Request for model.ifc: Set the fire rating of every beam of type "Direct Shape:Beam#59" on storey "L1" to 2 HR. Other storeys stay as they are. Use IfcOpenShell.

First a look at what the model holds.

```python
import ifcopenshell
import ifcopenshell.util.element

model = ifcopenshell.open("model.ifc")
print(model.schema)
storey = next(s for s in model.by_type("IfcBuildingStorey") if s.Name == "L1")
beams = [e for e in ifcopenshell.util.element.get_decomposition(storey) if e.is_a("IfcBeam")]
seen = {}
for e in beams:
    element_type = ifcopenshell.util.element.get_type(e)
    key = (element_type.Name if element_type != e and element_type else None, ifcopenshell.util.element.get_pset(e, "Pset_BeamCommon", "FireRating"))
    seen[key] = seen.get(key, 0) + 1
for (name, value), count in sorted(seen.items(), key=str):
    print(count, "x", name, "|", value)
```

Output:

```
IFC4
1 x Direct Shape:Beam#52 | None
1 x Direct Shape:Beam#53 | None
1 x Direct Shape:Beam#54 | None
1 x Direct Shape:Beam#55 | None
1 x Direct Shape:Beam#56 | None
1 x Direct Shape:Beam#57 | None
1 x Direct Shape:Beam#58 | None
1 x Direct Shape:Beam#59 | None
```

```python
import ifcopenshell
import ifcopenshell.api.pset
import ifcopenshell.util.element

model = ifcopenshell.open("model.ifc")

storey = next(s for s in model.by_type("IfcBuildingStorey") if s.Name == "L1")
beams = [e for e in ifcopenshell.util.element.get_decomposition(storey) if e.is_a("IfcBeam")]

count = 0
for e in beams:
    element_type = ifcopenshell.util.element.get_type(e)
    if element_type in (None, e) or element_type.Name != "Direct Shape:Beam#59":
        continue
    # add_pset returns the element's existing set when there is one.
    pset = ifcopenshell.api.pset.add_pset(model, product=e, name="Pset_BeamCommon")
    ifcopenshell.api.pset.edit_pset(model, pset=pset, properties={"FireRating": "2 HR"})
    count += 1

print(count, "beams updated")

model.write("model_v2.ifc")
```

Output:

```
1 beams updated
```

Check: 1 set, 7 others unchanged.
